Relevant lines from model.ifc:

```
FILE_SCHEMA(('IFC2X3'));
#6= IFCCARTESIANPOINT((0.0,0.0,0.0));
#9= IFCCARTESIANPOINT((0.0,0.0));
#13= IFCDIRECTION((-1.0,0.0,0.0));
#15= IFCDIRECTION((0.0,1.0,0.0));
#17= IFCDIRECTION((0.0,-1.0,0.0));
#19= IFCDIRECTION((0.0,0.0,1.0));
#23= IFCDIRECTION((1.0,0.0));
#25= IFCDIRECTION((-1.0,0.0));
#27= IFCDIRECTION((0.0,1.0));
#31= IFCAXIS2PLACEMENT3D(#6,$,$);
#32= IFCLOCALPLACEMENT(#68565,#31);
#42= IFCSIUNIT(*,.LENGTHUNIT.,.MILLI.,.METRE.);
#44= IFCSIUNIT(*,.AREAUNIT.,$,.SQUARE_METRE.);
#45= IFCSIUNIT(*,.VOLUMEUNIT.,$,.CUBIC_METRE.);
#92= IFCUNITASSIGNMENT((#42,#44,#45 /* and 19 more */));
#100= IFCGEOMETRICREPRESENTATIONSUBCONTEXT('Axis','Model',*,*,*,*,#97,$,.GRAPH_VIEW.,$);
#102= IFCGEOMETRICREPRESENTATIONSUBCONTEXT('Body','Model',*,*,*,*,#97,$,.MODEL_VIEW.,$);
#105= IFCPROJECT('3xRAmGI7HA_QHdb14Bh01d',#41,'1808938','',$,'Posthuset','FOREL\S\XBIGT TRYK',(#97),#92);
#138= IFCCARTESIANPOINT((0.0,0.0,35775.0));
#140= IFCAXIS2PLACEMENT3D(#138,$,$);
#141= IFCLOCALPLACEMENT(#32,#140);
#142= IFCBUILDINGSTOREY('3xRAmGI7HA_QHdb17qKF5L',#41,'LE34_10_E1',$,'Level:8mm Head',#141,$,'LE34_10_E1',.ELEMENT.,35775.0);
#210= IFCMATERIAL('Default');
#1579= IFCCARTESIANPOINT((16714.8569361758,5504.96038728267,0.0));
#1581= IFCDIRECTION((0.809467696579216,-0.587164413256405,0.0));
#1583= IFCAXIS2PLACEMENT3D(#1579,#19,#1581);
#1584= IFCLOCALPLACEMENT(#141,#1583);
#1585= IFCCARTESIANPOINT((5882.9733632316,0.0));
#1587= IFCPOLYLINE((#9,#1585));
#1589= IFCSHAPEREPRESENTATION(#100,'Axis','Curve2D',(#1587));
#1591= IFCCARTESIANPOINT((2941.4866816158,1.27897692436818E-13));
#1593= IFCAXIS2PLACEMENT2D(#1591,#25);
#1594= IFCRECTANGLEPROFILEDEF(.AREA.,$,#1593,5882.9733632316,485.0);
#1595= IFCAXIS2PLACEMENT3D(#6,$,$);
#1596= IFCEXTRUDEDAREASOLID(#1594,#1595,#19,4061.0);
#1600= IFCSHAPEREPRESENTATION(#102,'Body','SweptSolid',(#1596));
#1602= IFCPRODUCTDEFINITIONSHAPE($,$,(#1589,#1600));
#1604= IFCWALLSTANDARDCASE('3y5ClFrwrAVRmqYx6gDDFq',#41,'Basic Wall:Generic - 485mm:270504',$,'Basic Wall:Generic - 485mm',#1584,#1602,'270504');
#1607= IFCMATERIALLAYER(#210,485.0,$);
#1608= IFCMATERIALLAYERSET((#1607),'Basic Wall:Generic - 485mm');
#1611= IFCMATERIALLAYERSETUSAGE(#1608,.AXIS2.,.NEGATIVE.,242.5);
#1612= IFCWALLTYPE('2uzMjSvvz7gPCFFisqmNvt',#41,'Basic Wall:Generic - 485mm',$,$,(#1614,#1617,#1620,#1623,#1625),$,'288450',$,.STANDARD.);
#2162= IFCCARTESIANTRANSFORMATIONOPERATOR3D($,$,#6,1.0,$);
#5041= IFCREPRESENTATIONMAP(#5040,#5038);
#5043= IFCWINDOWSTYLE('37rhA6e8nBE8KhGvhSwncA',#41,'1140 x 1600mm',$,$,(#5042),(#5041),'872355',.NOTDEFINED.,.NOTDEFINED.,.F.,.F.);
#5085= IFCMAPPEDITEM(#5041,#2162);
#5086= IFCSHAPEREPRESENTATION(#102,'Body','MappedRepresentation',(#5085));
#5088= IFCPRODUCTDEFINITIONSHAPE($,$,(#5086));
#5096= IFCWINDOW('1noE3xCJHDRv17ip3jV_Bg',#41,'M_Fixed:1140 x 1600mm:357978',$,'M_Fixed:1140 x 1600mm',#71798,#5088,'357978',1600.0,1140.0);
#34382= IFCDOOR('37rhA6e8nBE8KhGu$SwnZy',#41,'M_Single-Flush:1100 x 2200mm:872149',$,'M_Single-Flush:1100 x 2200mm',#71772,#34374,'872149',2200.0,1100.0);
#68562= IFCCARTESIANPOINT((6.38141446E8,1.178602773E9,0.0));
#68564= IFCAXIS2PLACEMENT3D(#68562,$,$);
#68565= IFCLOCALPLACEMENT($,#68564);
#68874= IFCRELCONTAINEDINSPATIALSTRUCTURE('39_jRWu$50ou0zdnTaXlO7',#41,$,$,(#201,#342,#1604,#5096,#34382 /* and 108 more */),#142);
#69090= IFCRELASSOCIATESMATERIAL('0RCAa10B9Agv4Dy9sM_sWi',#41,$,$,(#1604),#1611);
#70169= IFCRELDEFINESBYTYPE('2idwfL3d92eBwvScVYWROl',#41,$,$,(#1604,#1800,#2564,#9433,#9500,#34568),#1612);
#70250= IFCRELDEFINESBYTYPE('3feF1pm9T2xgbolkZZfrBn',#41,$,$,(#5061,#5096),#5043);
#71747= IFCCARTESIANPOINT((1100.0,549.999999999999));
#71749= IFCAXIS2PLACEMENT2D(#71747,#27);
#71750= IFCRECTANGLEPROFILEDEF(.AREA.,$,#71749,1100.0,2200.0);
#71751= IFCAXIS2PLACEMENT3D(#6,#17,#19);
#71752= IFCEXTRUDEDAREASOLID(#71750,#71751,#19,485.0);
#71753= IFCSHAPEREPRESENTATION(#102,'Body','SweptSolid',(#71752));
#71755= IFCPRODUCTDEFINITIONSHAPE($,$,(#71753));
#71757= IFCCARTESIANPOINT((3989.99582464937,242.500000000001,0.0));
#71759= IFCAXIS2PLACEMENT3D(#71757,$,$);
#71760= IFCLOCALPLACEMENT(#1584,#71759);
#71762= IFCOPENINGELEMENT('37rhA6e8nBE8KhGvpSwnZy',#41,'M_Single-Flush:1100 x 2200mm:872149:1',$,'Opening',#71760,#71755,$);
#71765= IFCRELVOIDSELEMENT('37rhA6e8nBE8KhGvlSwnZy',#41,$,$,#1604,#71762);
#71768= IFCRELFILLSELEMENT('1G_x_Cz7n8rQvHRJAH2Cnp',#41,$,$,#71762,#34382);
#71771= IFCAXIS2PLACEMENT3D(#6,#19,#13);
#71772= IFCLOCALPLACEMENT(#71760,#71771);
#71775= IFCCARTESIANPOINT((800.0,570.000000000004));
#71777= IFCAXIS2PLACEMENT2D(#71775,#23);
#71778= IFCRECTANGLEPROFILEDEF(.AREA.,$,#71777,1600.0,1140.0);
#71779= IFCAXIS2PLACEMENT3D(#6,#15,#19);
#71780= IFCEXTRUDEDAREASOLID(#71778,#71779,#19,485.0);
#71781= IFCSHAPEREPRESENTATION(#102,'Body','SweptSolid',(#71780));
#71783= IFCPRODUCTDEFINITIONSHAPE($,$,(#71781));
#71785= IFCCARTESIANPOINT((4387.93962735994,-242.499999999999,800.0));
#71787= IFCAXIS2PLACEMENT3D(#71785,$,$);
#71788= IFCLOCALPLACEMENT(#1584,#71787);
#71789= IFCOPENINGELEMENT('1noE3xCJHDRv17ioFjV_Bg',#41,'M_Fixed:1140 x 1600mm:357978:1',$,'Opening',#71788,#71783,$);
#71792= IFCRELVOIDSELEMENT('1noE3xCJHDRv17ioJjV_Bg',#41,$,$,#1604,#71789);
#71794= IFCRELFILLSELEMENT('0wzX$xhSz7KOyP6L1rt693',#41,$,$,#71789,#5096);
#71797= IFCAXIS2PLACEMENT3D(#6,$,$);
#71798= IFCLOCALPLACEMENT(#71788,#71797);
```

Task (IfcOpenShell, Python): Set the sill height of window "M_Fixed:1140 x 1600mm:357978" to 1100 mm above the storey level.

```python
import numpy as np
import ifcopenshell
import ifcopenshell.api.geometry
import ifcopenshell.geom
import ifcopenshell.util.element
import ifcopenshell.util.placement
import ifcopenshell.util.shape
import ifcopenshell.util.unit

model = ifcopenshell.open("model.ifc")
unit_scale = ifcopenshell.util.unit.calculate_unit_scale(model)

window = model.by_guid("1noE3xCJHDRv17ip3jV_Bg")
opening = window.FillsVoids[0].RelatingOpeningElement
storey = ifcopenshell.util.element.get_container(window, ifc_class="IfcBuildingStorey")
level = ifcopenshell.util.placement.get_local_placement(storey.ObjectPlacement)[2, 3]

# The opening's origin need not be at the sill, so measure its lowest point.
shape = ifcopenshell.geom.create_shape(ifcopenshell.geom.settings(), opening)
bottom = ifcopenshell.util.shape.get_shape_bottom_elevation(shape, shape.geometry) / unit_scale
dz = level + 1100.0 - bottom

shift = np.array([0.0, 0.0, dz])
# The window is placed relative to its opening, so it follows when the opening moves.
matrix = ifcopenshell.util.placement.get_local_placement(opening.ObjectPlacement)
matrix[:3, 3] += shift
ifcopenshell.api.geometry.edit_object_placement(
    model, product=opening, matrix=matrix, is_si=False, should_transform_children=True
)

print(f"moved by {dz * unit_scale:+.3f} m")

model.write("model_v2.ifc")
```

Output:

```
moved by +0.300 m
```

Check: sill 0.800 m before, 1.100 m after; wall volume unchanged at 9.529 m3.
